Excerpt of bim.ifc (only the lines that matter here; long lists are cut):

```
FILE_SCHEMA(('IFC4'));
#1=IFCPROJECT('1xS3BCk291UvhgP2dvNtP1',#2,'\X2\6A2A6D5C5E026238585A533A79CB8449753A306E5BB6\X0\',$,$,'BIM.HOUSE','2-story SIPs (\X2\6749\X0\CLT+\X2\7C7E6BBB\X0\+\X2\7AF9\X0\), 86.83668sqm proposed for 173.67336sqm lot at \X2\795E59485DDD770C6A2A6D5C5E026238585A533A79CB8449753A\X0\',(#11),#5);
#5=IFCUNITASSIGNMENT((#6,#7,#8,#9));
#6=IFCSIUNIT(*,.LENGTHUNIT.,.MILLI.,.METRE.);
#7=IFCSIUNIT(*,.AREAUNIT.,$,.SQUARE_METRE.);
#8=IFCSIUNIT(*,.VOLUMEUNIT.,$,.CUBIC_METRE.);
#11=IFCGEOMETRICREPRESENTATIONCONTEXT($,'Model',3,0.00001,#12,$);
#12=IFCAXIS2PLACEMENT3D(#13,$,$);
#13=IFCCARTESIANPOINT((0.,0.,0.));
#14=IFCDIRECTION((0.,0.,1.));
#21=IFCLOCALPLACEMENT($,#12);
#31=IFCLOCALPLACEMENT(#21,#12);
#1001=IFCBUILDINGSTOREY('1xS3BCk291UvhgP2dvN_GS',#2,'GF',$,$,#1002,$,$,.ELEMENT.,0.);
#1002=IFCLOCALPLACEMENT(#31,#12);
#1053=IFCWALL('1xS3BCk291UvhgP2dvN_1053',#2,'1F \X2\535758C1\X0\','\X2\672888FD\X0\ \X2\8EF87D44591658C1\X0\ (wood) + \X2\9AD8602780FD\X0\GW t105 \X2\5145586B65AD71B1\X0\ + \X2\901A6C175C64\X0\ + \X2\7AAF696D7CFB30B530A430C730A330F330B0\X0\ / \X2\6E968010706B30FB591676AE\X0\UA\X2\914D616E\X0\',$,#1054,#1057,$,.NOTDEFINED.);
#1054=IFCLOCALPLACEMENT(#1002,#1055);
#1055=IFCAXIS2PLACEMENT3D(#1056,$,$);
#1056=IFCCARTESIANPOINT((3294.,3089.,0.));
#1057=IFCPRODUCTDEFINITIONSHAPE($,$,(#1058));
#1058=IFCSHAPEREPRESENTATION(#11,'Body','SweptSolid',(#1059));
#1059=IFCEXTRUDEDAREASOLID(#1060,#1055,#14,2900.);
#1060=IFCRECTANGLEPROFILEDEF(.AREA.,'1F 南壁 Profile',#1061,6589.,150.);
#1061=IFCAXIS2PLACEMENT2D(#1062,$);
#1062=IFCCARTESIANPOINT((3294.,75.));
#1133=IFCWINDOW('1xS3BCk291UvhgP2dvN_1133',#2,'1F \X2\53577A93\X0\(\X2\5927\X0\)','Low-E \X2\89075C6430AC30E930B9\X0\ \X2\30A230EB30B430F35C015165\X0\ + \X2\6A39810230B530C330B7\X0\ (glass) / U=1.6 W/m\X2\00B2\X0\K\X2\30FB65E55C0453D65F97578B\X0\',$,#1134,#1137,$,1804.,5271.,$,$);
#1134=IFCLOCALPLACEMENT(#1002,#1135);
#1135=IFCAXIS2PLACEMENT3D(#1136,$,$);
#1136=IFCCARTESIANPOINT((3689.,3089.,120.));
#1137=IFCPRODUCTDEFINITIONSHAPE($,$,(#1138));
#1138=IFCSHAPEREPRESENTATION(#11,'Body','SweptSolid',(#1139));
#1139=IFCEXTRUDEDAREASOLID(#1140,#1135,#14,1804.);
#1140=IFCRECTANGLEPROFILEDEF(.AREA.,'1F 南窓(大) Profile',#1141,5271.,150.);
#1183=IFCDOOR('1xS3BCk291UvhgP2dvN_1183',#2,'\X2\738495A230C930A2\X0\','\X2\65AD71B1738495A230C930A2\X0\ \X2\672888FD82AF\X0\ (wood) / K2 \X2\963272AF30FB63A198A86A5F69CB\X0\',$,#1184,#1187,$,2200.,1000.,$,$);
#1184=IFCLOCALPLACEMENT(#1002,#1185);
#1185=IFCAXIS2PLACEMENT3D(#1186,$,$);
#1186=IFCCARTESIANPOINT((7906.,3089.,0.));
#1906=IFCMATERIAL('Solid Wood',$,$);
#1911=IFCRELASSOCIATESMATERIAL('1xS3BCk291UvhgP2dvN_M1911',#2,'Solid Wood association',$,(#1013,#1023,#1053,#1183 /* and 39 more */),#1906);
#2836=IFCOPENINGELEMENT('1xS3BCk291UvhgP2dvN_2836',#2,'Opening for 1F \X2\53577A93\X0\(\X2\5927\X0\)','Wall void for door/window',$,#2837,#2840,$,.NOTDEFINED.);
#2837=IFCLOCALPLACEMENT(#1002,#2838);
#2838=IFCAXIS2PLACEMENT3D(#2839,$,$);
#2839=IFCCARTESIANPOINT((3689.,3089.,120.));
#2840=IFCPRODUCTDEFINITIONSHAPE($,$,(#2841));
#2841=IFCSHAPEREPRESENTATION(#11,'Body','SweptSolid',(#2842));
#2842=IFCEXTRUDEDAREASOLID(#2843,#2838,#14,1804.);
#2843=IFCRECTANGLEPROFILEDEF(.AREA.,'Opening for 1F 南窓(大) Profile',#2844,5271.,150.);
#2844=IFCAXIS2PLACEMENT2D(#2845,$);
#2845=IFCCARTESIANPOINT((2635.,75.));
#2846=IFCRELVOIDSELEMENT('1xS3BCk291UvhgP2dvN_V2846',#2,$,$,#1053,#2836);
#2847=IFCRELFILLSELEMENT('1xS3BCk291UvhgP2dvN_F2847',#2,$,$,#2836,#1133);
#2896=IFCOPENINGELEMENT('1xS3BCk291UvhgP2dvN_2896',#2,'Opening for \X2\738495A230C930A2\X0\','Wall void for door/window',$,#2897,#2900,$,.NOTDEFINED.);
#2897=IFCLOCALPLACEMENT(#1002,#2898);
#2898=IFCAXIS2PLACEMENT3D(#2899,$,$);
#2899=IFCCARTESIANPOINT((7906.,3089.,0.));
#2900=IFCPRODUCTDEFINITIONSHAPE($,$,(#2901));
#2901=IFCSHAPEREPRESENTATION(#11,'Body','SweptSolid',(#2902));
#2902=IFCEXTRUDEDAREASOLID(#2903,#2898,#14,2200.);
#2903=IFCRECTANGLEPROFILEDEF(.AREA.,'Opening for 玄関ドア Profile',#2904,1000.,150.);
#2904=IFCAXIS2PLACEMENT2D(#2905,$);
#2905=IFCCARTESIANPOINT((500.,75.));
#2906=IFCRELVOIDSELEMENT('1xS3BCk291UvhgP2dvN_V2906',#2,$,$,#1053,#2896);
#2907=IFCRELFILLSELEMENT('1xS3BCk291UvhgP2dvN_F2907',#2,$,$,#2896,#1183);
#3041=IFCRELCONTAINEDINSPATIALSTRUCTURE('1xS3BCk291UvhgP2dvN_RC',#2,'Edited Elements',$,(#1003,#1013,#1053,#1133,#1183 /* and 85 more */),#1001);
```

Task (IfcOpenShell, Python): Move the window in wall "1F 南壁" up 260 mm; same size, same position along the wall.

```python
import numpy as np
import ifcopenshell
import ifcopenshell.api.geometry
import ifcopenshell.util.placement
import ifcopenshell.util.unit

model = ifcopenshell.open("bim.ifc")
unit_scale = ifcopenshell.util.unit.calculate_unit_scale(model)

window = model.by_guid("1xS3BCk291UvhgP2dvN_1133")
opening = window.FillsVoids[0].RelatingOpeningElement
dz = 0.26 / unit_scale

shift = np.array([0.0, 0.0, dz])
# The window is not placed relative to its opening, so move both.
for product in (opening, window):
    matrix = ifcopenshell.util.placement.get_local_placement(product.ObjectPlacement)
    matrix[:3, 3] += shift
    ifcopenshell.api.geometry.edit_object_placement(model, product=product, matrix=matrix, is_si=False)

print(f"moved by {dz * unit_scale:+.3f} m")

model.write("bim_updated.ifc")
```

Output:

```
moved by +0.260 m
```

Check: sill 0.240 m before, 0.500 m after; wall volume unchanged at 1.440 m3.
